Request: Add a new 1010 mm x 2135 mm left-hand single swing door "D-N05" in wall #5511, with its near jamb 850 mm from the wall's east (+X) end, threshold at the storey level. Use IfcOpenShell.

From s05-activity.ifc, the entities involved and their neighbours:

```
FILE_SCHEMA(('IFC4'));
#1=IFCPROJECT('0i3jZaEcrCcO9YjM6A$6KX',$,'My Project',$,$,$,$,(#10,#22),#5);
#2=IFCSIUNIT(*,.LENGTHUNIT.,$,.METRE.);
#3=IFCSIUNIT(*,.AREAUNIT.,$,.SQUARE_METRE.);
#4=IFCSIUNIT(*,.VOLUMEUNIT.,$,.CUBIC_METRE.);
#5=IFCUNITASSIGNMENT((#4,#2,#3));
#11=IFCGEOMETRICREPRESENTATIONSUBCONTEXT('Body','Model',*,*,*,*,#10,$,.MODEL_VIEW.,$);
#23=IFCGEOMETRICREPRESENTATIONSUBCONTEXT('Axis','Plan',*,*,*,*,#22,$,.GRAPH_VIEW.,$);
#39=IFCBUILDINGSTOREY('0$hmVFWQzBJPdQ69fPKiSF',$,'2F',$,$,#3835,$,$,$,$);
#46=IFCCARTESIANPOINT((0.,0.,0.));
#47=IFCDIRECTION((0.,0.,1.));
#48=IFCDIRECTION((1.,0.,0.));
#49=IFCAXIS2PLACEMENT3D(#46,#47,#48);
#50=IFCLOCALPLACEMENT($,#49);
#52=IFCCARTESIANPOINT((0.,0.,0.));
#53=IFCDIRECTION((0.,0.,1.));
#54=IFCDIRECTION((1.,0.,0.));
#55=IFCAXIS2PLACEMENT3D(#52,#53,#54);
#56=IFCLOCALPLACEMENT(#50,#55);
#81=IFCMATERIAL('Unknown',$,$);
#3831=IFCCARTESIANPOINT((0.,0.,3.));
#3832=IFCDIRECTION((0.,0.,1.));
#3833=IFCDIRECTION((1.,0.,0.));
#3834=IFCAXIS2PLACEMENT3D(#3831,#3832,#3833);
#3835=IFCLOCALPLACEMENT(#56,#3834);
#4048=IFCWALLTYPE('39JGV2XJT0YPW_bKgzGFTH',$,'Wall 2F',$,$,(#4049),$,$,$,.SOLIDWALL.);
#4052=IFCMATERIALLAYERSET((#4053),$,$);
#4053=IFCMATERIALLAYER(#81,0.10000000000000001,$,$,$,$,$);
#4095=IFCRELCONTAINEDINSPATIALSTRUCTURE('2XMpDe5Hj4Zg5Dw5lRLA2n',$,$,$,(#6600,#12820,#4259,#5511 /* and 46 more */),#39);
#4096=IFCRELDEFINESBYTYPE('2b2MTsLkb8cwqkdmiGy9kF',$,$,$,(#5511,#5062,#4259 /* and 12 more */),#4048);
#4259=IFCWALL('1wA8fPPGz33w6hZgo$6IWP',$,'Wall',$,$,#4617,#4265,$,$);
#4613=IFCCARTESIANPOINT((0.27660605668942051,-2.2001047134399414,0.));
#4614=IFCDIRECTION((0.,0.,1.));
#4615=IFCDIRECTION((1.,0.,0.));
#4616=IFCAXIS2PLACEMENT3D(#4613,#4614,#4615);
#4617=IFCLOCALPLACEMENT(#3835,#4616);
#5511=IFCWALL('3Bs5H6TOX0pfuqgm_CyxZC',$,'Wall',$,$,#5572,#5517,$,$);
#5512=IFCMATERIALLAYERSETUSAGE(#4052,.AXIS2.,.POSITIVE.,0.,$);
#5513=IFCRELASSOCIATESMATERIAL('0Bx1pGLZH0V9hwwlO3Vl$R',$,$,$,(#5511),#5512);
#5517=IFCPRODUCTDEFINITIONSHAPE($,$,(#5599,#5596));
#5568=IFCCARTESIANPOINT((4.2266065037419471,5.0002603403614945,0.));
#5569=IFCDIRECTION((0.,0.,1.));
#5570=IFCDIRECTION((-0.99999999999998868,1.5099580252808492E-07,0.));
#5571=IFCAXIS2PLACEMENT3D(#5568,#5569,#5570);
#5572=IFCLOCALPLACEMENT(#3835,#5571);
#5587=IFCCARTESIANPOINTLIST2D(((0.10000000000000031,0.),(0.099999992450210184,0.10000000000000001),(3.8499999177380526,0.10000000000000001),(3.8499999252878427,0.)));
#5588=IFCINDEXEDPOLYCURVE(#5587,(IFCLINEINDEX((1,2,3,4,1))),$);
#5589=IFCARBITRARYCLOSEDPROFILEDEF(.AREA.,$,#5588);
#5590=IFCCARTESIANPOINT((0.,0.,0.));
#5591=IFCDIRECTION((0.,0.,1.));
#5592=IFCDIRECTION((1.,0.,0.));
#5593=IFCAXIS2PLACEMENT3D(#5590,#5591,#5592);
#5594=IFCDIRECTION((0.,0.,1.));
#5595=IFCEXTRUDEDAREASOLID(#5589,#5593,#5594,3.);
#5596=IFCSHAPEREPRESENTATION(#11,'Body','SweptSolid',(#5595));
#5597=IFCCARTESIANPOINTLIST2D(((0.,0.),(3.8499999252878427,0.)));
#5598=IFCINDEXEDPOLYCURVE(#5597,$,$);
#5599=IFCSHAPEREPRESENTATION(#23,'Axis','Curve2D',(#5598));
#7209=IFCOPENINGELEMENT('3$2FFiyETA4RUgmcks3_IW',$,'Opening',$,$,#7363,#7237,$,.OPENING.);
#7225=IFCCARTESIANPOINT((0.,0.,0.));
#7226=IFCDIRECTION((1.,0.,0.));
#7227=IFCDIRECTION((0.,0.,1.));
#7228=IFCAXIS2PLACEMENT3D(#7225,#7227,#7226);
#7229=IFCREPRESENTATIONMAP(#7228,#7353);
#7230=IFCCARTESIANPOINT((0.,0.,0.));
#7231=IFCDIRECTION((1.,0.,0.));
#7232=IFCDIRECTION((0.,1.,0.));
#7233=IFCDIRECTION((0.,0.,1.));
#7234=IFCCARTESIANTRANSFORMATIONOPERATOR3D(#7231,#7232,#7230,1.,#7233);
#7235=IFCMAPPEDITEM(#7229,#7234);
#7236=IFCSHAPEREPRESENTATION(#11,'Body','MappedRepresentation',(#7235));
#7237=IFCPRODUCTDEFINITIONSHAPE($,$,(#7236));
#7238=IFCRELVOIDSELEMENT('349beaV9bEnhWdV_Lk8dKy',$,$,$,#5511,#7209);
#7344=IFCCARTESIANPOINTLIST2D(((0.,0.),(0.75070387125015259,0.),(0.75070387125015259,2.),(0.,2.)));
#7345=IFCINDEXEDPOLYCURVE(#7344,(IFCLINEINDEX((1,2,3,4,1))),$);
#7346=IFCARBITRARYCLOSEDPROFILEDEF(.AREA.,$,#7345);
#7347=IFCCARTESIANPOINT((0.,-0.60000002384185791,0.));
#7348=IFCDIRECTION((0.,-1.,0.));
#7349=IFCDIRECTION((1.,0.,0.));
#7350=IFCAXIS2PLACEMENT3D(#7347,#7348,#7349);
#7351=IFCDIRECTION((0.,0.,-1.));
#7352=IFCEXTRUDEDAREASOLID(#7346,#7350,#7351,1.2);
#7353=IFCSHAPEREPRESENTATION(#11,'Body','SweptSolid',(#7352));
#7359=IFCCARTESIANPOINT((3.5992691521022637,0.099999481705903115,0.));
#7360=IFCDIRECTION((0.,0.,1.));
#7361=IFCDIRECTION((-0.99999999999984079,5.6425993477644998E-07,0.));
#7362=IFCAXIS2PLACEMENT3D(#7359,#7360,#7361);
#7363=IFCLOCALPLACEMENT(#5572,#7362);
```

```python
import numpy as np
import ifcopenshell
import ifcopenshell.api.feature
import ifcopenshell.api.geometry
import ifcopenshell.api.root
import ifcopenshell.api.spatial
import ifcopenshell.geom
import ifcopenshell.util.element
import ifcopenshell.util.placement
import ifcopenshell.util.representation
import ifcopenshell.util.shape
import ifcopenshell.util.unit

model = ifcopenshell.open("s05-activity.ifc")
unit_scale = ifcopenshell.util.unit.calculate_unit_scale(model)
settings = ifcopenshell.geom.settings()


def volume(element):
    """Net volume in cubic metres, openings subtracted."""
    shape = ifcopenshell.geom.create_shape(settings, element)
    return ifcopenshell.util.shape.get_volume(shape.geometry)


wall = model.by_id(5511)
storey = ifcopenshell.util.element.get_container(wall, ifc_class="IfcBuildingStorey")
context = ifcopenshell.util.representation.get_context(model, "Model", "Body", "MODEL_VIEW")
before = volume(wall)

width, height, from_end, sill = 1.01, 2.135, 0.85, 0.0  # metres

# The wall runs along its own X axis, and the end named is its -X end.
wall_shape = ifcopenshell.geom.create_shape(settings, wall)
x, y, z = ifcopenshell.util.shape.get_vertices(wall_shape.geometry).T
start = x.min() + from_end
face, thickness = float(y.min()), float(y.max() - y.min())
wall_matrix = ifcopenshell.util.placement.get_local_placement(wall.ObjectPlacement)
level = ifcopenshell.util.placement.get_local_placement(storey.ObjectPlacement)[2, 3]


def in_wall(x, y):
    """Placement at x, y metres in the wall's axes, at sill height."""
    matrix = wall_matrix.copy()
    matrix[:, 3] = wall_matrix @ np.array([x / unit_scale, y / unit_scale, 0.0, 1.0])
    matrix[2, 3] = level + sill / unit_scale
    return matrix


# Opening: a box that overshoots both wall faces by 50 mm.
opening = ifcopenshell.api.root.create_entity(model, ifc_class="IfcOpeningElement", predefined_type="OPENING")
box = ifcopenshell.api.geometry.add_wall_representation(
    model, context=context, length=width, height=height, thickness=thickness + 0.1
)
ifcopenshell.api.geometry.assign_representation(model, product=opening, representation=box)
ifcopenshell.api.geometry.edit_object_placement(model, product=opening, matrix=in_wall(start, face - 0.05), is_si=False)
ifcopenshell.api.feature.add_feature(model, feature=opening, element=wall)

door = ifcopenshell.api.root.create_entity(model, ifc_class="IfcDoor", name="D-N05", predefined_type="DOOR")
door.OverallWidth, door.OverallHeight = width / unit_scale, height / unit_scale
door.OperationType = "SINGLE_SWING_LEFT"
body = ifcopenshell.api.geometry.add_door_representation(
    model,
    context=context,
    overall_width=door.OverallWidth,
    overall_height=door.OverallHeight,
    operation_type="SINGLE_SWING_LEFT",
    lining_properties={"LiningDepth": thickness / unit_scale, "ThresholdDepth": thickness / unit_scale},
)
ifcopenshell.api.geometry.assign_representation(model, product=door, representation=body)
ifcopenshell.api.spatial.assign_container(model, products=[door], relating_structure=storey)
ifcopenshell.api.feature.add_filling(model, opening=opening, element=door)

# The lining spans the wall, so the door starts at the wall face.
ifcopenshell.api.geometry.edit_object_placement(model, product=door, matrix=in_wall(start, face), is_si=False)

after = volume(wall)

print(f"wall volume {before:.3f} -> {after:.3f} m3")

model.write("s05-activity_updated.ifc")
```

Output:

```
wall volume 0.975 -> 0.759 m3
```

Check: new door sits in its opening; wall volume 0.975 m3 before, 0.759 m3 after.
